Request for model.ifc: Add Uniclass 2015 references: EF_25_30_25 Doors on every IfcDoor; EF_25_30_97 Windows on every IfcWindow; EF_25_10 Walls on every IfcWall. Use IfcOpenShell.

First a look at what the model holds.

```python
import ifcopenshell

model = ifcopenshell.open("model.ifc")
print(model.schema)
print("classifications:", [c.Name for c in model.by_type("IfcClassification")])
for ifc_class in ("IfcDoor", "IfcRoof", "IfcStair", "IfcWall", "IfcWindow"):
    print(ifc_class, len(model.by_type(ifc_class)))
```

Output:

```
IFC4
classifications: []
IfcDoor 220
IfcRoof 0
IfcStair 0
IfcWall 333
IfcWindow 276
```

```python
import ifcopenshell
import ifcopenshell.api.classification

model = ifcopenshell.open("model.ifc")

system = ifcopenshell.api.classification.add_classification(model, classification="Uniclass 2015")

codes = {
    "IfcDoor": ("EF_25_30_25", "Doors"),
    "IfcWindow": ("EF_25_30_97", "Windows"),
    "IfcWall": ("EF_25_10", "Walls"),
}
for ifc_class, (code, name) in codes.items():
    products = model.by_type(ifc_class)
    ifcopenshell.api.classification.add_reference(
        model, products=products, classification=system, identification=code, name=name
    )
    print(code, len(products))

model.write("model_v2.ifc")
```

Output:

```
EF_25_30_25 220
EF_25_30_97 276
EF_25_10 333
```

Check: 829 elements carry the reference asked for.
